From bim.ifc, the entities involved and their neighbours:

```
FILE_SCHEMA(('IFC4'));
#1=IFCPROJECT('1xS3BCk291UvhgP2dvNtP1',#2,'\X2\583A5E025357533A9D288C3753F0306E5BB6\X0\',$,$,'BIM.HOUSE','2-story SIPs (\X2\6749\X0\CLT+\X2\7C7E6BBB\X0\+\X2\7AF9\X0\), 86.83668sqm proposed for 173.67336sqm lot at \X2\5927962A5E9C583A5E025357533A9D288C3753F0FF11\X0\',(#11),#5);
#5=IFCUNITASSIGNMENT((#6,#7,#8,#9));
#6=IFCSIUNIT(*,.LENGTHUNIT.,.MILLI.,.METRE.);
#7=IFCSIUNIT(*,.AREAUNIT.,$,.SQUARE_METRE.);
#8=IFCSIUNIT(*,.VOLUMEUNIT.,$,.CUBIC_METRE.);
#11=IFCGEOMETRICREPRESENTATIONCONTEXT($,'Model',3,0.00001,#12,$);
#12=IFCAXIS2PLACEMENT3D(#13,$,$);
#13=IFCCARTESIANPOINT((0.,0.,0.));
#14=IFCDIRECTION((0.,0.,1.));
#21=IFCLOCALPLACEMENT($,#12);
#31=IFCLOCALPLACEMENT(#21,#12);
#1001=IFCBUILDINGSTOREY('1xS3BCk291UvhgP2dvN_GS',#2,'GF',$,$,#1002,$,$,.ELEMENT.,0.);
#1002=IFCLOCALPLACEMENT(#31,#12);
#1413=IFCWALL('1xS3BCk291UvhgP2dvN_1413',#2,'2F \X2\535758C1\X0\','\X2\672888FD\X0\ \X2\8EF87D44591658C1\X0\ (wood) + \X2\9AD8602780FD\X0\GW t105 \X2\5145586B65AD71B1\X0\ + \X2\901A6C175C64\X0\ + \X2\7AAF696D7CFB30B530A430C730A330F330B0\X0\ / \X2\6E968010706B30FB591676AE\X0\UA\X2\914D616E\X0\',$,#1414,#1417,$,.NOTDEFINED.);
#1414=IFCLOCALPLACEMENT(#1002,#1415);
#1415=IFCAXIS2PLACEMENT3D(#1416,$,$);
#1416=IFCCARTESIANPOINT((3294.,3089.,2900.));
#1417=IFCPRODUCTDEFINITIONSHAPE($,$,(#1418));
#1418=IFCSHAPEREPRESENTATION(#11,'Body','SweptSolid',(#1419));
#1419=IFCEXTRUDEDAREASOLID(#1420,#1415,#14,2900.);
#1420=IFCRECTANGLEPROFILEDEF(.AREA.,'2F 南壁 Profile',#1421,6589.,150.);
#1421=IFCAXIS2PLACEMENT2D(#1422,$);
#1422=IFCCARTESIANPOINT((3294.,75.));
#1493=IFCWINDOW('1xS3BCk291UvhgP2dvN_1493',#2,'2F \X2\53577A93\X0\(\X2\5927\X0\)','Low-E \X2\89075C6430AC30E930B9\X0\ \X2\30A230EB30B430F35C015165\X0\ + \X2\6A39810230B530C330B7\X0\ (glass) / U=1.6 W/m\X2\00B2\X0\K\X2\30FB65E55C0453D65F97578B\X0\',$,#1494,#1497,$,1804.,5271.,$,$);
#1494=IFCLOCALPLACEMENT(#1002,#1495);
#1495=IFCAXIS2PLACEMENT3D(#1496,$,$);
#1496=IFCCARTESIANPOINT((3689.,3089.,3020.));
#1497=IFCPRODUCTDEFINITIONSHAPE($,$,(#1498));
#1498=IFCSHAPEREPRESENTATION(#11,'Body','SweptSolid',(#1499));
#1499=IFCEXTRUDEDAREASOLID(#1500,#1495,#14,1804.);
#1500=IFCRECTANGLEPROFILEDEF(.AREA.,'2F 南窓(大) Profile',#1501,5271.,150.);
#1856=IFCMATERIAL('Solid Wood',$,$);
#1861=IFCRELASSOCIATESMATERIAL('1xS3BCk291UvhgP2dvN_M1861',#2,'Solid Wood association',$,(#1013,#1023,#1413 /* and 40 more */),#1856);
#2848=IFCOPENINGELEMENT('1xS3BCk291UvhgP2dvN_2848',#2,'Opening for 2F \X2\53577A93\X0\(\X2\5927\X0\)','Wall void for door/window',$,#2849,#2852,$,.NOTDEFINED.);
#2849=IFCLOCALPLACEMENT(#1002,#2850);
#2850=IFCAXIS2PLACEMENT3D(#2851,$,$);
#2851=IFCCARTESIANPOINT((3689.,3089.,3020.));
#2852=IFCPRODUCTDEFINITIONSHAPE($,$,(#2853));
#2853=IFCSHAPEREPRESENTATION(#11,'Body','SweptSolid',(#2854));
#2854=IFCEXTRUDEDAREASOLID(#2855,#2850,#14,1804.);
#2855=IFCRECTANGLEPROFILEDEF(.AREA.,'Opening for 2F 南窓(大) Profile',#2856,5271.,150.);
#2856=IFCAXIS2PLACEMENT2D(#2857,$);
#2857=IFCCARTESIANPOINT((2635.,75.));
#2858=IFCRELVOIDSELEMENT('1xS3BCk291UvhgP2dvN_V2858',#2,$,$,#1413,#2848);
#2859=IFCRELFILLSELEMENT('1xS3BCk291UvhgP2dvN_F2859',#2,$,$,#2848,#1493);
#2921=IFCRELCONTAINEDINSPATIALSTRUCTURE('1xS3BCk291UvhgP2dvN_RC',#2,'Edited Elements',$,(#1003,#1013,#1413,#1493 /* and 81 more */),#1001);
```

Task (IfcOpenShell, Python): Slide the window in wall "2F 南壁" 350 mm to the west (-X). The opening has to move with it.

```python
import ifcopenshell
import ifcopenshell.api.geometry
import ifcopenshell.util.placement

model = ifcopenshell.open("bim.ifc")

window = model.by_guid("1xS3BCk291UvhgP2dvN_1493")
opening = window.FillsVoids[0].RelatingOpeningElement
wall = opening.VoidsElements[0].RelatingBuildingElement

wall_matrix = ifcopenshell.util.placement.get_local_placement(wall.ObjectPlacement)
shift = wall_matrix[:3, 0] * -350.0
before = ifcopenshell.util.placement.get_local_placement(window.ObjectPlacement)[:3, 3].copy()

# The window is not placed relative to its opening, so move both.
for product in (opening, window):
    matrix = ifcopenshell.util.placement.get_local_placement(product.ObjectPlacement)
    matrix[:3, 3] += shift
    ifcopenshell.api.geometry.edit_object_placement(model, product=product, matrix=matrix, is_si=False)

after = ifcopenshell.util.placement.get_local_placement(window.ObjectPlacement)[:3, 3]
print("window moved by", (after - before).round(3) + 0.0)

model.write("bim_rev.ifc")
```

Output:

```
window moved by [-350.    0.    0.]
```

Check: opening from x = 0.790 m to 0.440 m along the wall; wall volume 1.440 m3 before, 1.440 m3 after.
